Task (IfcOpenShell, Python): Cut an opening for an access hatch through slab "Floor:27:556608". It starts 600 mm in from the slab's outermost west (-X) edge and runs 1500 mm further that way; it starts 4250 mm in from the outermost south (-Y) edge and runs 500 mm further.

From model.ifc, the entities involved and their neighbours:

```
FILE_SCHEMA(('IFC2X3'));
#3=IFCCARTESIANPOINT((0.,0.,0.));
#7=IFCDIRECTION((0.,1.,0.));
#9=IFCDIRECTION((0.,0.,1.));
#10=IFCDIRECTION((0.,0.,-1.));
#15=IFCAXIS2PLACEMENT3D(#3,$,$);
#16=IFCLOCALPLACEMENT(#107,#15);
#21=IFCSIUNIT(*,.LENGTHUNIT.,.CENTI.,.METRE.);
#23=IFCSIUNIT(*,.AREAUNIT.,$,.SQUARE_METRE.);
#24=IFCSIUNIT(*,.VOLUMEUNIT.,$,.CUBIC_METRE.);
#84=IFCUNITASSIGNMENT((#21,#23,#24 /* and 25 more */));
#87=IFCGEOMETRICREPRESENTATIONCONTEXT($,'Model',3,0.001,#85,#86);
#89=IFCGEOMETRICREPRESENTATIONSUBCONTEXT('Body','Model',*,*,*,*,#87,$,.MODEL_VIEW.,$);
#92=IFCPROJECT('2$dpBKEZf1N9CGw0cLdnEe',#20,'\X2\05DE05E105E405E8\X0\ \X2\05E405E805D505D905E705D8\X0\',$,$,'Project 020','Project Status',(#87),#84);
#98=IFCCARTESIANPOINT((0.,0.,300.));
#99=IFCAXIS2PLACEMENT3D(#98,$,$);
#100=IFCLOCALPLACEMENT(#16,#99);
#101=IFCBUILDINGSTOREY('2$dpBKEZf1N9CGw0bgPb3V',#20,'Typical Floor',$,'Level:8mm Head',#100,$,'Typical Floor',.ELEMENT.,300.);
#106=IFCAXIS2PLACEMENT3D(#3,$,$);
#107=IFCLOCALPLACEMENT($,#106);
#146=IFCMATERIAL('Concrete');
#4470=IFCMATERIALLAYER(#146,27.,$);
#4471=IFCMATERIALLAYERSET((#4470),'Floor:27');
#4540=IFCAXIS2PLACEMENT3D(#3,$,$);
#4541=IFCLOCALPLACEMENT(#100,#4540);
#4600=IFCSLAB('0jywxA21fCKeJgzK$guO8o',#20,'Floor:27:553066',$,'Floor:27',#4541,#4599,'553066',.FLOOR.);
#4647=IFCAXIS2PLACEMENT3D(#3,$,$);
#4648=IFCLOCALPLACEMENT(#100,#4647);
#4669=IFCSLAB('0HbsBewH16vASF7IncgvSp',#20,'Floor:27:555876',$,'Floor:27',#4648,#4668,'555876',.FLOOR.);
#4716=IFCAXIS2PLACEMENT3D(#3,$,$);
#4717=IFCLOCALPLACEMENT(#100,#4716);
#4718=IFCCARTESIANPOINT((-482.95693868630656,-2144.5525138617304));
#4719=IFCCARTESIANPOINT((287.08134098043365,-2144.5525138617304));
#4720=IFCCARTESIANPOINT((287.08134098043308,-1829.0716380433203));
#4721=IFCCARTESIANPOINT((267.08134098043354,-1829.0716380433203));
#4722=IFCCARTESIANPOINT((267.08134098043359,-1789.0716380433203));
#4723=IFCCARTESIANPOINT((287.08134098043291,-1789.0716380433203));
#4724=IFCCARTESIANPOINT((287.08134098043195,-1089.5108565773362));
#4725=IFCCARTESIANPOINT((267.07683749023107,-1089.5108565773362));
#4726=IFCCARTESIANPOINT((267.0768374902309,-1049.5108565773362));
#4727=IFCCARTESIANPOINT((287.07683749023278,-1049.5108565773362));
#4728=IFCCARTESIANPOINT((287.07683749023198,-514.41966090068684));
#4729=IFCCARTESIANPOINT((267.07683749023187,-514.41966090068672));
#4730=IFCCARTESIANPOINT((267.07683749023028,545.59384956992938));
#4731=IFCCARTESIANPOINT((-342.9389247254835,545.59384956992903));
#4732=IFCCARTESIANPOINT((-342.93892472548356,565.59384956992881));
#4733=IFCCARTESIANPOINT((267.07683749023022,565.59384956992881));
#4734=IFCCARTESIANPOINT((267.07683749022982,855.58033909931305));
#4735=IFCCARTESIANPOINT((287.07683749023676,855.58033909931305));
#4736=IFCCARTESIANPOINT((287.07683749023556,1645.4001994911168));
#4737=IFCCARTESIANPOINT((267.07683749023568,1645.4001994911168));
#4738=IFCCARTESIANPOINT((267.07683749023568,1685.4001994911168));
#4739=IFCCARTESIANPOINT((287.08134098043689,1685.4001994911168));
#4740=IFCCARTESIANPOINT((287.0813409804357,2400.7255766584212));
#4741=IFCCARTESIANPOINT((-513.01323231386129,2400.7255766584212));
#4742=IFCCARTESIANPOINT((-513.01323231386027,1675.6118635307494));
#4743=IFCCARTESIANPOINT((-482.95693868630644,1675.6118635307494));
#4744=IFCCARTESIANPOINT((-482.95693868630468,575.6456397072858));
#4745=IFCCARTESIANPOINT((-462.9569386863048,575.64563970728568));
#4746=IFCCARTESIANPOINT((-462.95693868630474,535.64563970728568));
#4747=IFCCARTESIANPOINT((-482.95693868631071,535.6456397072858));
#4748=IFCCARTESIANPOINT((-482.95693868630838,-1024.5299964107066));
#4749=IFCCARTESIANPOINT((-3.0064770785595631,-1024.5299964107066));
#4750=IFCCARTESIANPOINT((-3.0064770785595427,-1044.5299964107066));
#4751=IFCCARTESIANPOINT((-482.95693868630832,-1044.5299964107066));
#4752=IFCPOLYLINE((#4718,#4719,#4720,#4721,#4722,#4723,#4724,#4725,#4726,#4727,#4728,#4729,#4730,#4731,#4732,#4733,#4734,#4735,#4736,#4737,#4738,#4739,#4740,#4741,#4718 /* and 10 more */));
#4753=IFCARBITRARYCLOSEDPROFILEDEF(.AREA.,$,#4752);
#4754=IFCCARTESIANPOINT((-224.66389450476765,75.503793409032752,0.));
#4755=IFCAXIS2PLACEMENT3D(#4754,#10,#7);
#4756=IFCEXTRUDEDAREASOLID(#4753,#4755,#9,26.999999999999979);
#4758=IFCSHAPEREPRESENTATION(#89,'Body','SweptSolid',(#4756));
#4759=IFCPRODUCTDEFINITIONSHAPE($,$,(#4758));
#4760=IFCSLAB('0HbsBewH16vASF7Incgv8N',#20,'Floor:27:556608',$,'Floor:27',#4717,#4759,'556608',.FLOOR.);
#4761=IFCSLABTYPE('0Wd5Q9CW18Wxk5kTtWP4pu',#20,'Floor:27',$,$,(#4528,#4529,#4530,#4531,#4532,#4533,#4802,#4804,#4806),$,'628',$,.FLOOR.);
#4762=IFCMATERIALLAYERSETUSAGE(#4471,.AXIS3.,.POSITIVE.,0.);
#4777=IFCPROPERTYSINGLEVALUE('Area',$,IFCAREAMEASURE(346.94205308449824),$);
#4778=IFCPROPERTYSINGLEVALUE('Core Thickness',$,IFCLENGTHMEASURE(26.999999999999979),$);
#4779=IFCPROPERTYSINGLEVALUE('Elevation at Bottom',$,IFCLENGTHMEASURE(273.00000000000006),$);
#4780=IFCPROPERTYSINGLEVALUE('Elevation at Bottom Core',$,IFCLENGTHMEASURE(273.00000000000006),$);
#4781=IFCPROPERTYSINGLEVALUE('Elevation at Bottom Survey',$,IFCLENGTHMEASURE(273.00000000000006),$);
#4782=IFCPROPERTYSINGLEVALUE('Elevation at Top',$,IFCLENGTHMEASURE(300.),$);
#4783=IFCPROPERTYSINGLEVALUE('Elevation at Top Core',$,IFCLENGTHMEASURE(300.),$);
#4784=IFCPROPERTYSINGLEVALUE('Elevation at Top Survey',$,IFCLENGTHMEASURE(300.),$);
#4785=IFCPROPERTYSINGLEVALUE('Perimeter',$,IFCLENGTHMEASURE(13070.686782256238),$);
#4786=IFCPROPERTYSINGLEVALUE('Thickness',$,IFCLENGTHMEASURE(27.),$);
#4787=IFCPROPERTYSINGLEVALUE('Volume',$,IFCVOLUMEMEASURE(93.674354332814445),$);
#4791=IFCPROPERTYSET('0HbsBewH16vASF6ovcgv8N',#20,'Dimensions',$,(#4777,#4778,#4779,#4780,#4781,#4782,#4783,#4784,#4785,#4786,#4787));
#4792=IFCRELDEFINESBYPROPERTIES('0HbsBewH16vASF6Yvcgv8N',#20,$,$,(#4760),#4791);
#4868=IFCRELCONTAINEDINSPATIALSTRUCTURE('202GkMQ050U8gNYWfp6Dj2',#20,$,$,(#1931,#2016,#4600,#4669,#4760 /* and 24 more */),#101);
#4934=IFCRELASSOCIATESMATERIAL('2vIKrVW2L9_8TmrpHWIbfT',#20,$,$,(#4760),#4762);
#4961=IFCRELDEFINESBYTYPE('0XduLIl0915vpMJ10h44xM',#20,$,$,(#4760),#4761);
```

```python
import numpy as np
import ifcopenshell
import ifcopenshell.api.feature
import ifcopenshell.api.geometry
import ifcopenshell.api.pset
import ifcopenshell.api.root
import ifcopenshell.geom
import ifcopenshell.util.element
import ifcopenshell.util.placement
import ifcopenshell.util.representation
import ifcopenshell.util.shape
import ifcopenshell.util.unit

model = ifcopenshell.open("model.ifc")
unit_scale = ifcopenshell.util.unit.calculate_unit_scale(model)
area_scale = ifcopenshell.util.unit.calculate_unit_scale(model, "AREAUNIT")
volume_scale = ifcopenshell.util.unit.calculate_unit_scale(model, "VOLUMEUNIT")
settings = ifcopenshell.geom.settings()


def volume(element):
    """Net volume in cubic metres, openings subtracted."""
    shape = ifcopenshell.geom.create_shape(settings, element)
    return ifcopenshell.util.shape.get_volume(shape.geometry)


slab = model.by_id(4760)
before = volume(slab)

# Extent in the slab's own axes, in metres. The edges named are its -X and -Y sides.
slab_shape = ifcopenshell.geom.create_shape(settings, slab)
vertices = ifcopenshell.util.shape.get_vertices(slab_shape.geometry)
x_min, y_min, bottom = vertices.min(axis=0)
top = vertices[:, 2].max()

opening = ifcopenshell.api.root.create_entity(model, ifc_class="IfcOpeningElement", name="Access hatch opening")
context = ifcopenshell.util.representation.get_context(model, "Model", "Body", "MODEL_VIEW")
width, depth = 1.5, 0.5
outline = [(0.0, 0.0), (width, 0.0), (width, depth), (0.0, depth), (0.0, 0.0)]
# Overshoot both faces by 50 mm so the cut is clean.
shape = ifcopenshell.api.geometry.add_slab_representation(
    model, context=context, depth=top - bottom + 0.1, polyline=outline
)
ifcopenshell.api.geometry.assign_representation(model, product=opening, representation=shape)

matrix = ifcopenshell.util.placement.get_local_placement(slab.ObjectPlacement)
matrix[:, 3] = matrix @ np.append(np.array([x_min + 0.6, y_min + 4.25, bottom - 0.05]) / unit_scale, 1.0)
ifcopenshell.api.geometry.edit_object_placement(model, product=opening, matrix=matrix, is_si=False)
ifcopenshell.api.feature.add_feature(model, feature=opening, element=slab)

after = volume(slab)

# Update the slab's stored quantities.
pset = model.by_id(ifcopenshell.util.element.get_pset(slab, "Dimensions", should_inherit=False)["id"])
ifcopenshell.api.pset.edit_pset(model, pset=pset, properties={
    "Area": model.create_entity("IfcAreaMeasure", after / (top - bottom) / area_scale),
    "Volume": model.create_entity("IfcVolumeMeasure", after / volume_scale),
})

print(f"slab volume {before:.3f} -> {after:.3f} m3")

model.write("model_updated.ifc")
```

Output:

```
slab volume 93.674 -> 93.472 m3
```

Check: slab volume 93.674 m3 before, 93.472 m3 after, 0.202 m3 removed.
